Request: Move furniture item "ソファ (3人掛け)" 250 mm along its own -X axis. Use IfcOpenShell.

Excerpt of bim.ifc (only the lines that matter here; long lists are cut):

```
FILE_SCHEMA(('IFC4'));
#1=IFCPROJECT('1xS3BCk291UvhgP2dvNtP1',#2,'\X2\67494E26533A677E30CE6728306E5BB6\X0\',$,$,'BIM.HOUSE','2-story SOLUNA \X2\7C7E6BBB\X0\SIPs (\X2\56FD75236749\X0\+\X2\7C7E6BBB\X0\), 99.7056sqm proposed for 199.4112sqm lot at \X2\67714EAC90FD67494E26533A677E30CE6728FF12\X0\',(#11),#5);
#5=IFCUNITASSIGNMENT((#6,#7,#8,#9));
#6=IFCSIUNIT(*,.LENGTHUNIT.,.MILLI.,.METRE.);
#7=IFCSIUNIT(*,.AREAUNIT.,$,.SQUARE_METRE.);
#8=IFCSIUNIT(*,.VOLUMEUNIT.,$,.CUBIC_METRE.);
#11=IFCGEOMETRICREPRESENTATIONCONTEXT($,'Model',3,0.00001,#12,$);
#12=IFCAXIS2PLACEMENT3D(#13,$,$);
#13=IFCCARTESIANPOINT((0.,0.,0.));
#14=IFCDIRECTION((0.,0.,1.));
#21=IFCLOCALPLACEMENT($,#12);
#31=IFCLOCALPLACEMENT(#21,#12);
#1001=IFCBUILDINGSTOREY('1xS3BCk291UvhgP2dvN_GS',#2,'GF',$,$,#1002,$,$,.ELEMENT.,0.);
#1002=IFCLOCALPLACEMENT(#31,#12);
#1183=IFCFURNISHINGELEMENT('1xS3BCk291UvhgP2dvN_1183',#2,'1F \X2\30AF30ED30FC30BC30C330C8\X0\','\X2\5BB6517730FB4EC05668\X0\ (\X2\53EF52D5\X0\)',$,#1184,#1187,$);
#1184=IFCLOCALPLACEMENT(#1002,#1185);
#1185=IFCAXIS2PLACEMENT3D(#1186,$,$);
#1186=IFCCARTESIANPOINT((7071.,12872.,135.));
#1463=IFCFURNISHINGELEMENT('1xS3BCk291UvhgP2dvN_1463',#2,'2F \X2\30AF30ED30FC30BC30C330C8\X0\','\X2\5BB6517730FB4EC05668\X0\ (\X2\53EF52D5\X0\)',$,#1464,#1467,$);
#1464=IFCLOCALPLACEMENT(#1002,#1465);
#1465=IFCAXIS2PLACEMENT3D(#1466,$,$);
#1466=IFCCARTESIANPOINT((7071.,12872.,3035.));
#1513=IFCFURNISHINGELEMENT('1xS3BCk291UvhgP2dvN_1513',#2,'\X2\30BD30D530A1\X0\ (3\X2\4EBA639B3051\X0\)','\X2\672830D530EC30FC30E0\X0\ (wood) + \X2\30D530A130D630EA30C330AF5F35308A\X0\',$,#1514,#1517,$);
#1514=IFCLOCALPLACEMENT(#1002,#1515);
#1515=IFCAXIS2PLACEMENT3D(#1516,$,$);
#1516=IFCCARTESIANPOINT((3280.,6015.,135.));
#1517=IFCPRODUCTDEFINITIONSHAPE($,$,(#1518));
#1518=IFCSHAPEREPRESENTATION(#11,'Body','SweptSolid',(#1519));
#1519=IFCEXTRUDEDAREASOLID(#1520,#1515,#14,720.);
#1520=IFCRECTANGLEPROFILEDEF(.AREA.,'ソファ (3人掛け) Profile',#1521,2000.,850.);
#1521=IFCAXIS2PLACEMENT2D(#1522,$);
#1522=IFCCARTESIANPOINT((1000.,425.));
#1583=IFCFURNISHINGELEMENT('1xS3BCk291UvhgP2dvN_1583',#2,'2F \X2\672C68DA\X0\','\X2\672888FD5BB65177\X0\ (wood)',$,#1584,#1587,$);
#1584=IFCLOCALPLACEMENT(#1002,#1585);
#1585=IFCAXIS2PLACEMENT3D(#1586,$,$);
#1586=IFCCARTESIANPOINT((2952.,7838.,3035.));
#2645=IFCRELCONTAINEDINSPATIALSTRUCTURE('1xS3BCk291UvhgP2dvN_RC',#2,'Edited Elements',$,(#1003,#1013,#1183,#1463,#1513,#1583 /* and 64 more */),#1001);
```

```python
import ifcopenshell
import ifcopenshell.api.geometry
import ifcopenshell.util.placement
import ifcopenshell.util.unit

model = ifcopenshell.open("bim.ifc")
unit_scale = ifcopenshell.util.unit.calculate_unit_scale(model)

item = model.by_id(1513)
matrix = ifcopenshell.util.placement.get_local_placement(item.ObjectPlacement)
matrix[:3, 3] -= matrix[:3, 0] * 0.25 / unit_scale
ifcopenshell.api.geometry.edit_object_placement(model, product=item, matrix=matrix, is_si=False)

print(ifcopenshell.util.placement.get_local_placement(item.ObjectPlacement).round(3) + 0.0)

model.write("bim_updated.ifc")
```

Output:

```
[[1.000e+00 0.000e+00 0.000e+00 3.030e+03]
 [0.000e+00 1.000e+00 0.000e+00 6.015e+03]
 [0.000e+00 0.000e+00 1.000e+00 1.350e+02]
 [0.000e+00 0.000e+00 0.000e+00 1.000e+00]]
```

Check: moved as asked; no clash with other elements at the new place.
